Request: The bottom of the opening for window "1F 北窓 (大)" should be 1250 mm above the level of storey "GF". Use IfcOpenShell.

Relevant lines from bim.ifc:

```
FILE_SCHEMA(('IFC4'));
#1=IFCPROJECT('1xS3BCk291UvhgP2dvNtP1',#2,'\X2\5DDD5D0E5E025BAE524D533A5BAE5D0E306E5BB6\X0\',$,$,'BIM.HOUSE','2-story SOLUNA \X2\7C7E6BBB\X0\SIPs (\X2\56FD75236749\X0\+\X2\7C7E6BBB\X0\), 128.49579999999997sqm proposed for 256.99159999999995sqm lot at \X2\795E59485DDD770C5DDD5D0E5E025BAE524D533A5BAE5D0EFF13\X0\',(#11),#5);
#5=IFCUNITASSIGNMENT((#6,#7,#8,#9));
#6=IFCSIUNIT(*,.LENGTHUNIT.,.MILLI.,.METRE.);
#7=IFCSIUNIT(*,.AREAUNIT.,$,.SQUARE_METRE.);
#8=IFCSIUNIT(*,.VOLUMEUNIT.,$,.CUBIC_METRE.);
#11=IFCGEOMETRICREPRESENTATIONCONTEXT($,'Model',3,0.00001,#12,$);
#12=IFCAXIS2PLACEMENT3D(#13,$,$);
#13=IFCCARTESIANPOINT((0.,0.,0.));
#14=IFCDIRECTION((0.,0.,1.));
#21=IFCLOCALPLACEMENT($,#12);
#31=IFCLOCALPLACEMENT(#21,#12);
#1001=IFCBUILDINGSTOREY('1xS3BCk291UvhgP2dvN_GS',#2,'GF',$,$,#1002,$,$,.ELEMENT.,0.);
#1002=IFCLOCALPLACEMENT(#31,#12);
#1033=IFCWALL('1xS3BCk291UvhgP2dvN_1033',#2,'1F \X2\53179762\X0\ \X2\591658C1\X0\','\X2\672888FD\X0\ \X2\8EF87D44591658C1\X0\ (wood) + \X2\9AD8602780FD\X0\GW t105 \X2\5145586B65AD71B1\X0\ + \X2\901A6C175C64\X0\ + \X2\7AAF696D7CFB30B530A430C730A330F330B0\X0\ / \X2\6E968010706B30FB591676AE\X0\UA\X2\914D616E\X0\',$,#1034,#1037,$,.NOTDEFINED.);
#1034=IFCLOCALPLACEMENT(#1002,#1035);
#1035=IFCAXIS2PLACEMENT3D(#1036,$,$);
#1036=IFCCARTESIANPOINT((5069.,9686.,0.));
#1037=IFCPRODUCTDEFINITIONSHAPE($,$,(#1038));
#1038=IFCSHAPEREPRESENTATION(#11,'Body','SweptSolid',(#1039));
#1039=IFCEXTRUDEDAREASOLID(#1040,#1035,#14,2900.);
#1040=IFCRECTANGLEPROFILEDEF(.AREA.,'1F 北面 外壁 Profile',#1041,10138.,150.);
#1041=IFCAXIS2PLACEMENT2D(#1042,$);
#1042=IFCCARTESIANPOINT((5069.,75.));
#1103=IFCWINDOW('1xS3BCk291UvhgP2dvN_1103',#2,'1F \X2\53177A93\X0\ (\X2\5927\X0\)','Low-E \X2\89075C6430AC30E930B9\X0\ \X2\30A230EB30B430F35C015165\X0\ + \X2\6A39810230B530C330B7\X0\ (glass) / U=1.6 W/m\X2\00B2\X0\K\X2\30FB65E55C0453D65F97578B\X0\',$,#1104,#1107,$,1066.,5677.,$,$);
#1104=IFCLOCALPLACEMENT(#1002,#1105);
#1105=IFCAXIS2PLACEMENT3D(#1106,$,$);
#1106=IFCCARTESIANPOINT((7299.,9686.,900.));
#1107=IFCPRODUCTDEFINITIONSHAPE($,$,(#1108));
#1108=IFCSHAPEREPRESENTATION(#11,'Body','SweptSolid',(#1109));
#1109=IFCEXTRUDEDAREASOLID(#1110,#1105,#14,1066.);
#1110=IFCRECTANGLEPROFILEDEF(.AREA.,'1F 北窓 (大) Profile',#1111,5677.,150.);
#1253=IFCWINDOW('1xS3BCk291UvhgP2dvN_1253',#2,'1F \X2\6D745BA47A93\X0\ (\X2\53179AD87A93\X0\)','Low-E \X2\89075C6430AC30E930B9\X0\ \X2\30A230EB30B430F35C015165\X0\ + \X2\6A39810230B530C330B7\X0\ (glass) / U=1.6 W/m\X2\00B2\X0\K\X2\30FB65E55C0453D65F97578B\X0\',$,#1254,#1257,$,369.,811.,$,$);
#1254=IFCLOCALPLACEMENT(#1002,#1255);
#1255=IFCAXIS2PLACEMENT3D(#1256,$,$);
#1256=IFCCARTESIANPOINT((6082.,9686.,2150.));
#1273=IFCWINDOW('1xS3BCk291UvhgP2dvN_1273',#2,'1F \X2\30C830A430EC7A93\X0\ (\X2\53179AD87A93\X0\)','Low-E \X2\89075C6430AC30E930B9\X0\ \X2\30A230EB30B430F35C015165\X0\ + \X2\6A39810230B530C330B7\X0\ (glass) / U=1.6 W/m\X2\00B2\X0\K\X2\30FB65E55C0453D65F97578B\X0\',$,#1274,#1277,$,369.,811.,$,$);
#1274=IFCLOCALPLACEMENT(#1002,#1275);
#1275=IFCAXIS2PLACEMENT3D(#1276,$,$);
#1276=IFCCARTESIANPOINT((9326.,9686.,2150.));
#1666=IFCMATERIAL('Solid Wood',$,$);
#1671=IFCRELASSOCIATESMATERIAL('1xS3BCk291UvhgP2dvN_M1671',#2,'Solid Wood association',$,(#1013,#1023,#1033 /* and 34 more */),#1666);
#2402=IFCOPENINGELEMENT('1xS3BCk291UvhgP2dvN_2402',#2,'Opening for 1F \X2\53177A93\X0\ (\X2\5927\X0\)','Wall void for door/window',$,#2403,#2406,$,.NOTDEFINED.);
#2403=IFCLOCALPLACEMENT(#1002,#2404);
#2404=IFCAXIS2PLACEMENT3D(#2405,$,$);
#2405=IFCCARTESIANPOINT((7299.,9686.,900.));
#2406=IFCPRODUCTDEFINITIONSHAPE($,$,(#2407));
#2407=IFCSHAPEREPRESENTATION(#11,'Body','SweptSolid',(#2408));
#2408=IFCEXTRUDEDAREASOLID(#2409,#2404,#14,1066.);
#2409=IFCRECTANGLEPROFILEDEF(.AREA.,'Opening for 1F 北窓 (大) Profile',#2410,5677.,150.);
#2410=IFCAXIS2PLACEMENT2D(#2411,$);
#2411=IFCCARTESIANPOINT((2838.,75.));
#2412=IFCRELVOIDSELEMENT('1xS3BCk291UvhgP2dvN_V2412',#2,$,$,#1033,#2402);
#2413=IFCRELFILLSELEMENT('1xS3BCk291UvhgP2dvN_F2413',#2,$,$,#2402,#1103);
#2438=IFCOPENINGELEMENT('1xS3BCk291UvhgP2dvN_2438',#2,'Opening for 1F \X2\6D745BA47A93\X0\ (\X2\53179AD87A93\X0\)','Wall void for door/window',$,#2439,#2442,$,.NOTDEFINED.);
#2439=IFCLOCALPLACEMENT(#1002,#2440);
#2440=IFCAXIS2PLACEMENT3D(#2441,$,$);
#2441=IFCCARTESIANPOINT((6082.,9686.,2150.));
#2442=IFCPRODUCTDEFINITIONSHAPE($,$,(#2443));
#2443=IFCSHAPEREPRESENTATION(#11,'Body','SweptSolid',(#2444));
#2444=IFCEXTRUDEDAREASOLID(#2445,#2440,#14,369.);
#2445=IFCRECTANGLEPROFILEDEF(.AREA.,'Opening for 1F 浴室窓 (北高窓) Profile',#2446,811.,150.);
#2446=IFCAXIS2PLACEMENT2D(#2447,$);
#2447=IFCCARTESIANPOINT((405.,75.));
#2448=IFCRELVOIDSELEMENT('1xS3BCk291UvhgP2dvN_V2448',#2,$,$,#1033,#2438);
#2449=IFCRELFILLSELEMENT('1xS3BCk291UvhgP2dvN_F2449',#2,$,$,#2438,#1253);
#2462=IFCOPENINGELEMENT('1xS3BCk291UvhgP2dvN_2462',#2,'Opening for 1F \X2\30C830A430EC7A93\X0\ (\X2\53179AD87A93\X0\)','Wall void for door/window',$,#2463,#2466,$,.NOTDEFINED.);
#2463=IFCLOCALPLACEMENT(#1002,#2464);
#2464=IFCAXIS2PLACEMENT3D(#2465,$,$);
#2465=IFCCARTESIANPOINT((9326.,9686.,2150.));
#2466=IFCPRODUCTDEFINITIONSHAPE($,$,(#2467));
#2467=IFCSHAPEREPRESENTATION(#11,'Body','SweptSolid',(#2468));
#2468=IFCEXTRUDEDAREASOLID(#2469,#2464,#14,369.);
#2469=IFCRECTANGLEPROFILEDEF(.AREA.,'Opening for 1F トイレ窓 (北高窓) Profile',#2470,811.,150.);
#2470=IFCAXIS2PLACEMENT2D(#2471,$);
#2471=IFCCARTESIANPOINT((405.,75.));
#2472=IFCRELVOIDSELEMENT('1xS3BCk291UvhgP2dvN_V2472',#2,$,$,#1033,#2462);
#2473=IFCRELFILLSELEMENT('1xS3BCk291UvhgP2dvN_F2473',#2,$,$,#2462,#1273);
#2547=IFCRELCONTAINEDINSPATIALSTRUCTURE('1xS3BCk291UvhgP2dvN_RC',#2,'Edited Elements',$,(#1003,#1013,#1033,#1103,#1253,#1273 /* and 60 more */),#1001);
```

```python
import numpy as np
import ifcopenshell
import ifcopenshell.api.geometry
import ifcopenshell.geom
import ifcopenshell.util.element
import ifcopenshell.util.placement
import ifcopenshell.util.shape
import ifcopenshell.util.unit

model = ifcopenshell.open("bim.ifc")
unit_scale = ifcopenshell.util.unit.calculate_unit_scale(model)

window = model.by_guid("1xS3BCk291UvhgP2dvN_1103")
opening = window.FillsVoids[0].RelatingOpeningElement
storey = ifcopenshell.util.element.get_container(window, ifc_class="IfcBuildingStorey")
level = ifcopenshell.util.placement.get_local_placement(storey.ObjectPlacement)[2, 3]

# The opening's origin need not be at the sill, so measure its lowest point.
shape = ifcopenshell.geom.create_shape(ifcopenshell.geom.settings(), opening)
bottom = ifcopenshell.util.shape.get_shape_bottom_elevation(shape, shape.geometry) / unit_scale
dz = level + 1.25 / unit_scale - bottom

shift = np.array([0.0, 0.0, dz])
# The window is not placed relative to its opening, so move both.
for product in (opening, window):
    matrix = ifcopenshell.util.placement.get_local_placement(product.ObjectPlacement)
    matrix[:3, 3] += shift
    ifcopenshell.api.geometry.edit_object_placement(model, product=product, matrix=matrix, is_si=False)

print(f"moved by {dz * unit_scale:+.3f} m")

model.write("bim_v2.ifc")
```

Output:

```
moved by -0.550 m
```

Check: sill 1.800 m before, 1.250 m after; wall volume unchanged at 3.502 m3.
